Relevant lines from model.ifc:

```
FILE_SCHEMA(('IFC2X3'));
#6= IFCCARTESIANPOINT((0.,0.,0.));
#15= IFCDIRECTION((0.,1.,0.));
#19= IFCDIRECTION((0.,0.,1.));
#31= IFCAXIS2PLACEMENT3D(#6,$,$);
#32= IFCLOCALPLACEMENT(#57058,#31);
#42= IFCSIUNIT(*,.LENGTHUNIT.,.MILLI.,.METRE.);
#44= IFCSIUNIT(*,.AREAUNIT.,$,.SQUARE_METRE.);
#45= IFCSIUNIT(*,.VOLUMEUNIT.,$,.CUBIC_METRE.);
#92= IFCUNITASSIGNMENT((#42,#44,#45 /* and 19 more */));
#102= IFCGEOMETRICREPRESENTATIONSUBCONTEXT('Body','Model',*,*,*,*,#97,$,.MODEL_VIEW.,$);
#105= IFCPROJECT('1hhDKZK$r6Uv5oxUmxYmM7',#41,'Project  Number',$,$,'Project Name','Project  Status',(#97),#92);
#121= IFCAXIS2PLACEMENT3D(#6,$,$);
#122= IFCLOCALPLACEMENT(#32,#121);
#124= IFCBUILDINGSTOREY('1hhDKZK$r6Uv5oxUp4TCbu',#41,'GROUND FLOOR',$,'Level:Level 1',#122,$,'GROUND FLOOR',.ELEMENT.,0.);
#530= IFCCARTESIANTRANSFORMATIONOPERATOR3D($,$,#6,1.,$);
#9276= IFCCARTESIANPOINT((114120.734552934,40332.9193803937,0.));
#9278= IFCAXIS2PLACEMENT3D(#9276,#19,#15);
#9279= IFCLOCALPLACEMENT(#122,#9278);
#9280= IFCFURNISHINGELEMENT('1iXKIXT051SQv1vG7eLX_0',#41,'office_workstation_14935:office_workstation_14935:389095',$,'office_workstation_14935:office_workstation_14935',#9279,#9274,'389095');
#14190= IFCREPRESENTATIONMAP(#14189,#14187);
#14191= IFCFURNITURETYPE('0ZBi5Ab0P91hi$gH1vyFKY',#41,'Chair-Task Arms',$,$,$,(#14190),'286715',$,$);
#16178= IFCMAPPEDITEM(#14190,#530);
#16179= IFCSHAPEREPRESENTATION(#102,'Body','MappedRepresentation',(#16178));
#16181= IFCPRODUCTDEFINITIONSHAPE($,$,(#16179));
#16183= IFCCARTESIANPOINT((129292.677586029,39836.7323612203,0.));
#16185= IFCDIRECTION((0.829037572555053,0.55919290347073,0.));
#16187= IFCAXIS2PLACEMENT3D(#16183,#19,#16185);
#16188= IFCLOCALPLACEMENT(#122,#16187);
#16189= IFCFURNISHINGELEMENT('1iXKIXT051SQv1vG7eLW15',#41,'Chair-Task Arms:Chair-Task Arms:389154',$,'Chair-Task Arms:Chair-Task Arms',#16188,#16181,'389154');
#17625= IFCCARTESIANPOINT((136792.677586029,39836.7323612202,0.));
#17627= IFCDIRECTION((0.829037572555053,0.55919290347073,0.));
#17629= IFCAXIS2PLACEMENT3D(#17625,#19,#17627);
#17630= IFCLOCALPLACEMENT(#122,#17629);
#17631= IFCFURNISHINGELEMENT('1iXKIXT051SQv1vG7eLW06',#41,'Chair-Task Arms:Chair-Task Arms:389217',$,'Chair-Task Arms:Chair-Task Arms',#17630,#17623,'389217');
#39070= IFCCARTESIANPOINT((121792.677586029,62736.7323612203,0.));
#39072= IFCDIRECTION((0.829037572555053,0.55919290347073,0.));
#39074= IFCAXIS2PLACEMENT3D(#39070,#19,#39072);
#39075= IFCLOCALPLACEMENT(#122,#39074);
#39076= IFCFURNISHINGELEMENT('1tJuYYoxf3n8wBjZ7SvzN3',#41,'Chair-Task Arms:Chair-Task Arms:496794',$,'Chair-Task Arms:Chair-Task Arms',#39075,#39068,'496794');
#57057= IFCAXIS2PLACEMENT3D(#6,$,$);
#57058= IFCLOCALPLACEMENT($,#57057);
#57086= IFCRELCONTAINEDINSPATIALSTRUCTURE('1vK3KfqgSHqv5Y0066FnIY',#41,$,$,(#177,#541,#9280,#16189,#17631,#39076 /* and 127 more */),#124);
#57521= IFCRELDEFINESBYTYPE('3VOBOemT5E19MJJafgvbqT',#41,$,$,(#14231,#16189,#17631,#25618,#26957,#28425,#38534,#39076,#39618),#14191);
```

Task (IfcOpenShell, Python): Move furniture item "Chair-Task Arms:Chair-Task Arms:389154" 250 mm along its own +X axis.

```python
import ifcopenshell
import ifcopenshell.api.geometry
import ifcopenshell.util.placement

model = ifcopenshell.open("model.ifc")

item = model.by_guid("1iXKIXT051SQv1vG7eLW15")
matrix = ifcopenshell.util.placement.get_local_placement(item.ObjectPlacement)
matrix[:3, 3] += matrix[:3, 0] * 250.0
ifcopenshell.api.geometry.edit_object_placement(model, product=item, matrix=matrix, is_si=False)

print(ifcopenshell.util.placement.get_local_placement(item.ObjectPlacement).round(3) + 0.0)

model.write("model-out.ifc")
```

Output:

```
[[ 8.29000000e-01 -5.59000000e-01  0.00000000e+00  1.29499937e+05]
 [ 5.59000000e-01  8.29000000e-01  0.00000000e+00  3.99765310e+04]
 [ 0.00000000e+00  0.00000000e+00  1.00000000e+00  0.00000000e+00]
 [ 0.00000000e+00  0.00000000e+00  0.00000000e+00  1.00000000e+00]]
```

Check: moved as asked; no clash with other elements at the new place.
